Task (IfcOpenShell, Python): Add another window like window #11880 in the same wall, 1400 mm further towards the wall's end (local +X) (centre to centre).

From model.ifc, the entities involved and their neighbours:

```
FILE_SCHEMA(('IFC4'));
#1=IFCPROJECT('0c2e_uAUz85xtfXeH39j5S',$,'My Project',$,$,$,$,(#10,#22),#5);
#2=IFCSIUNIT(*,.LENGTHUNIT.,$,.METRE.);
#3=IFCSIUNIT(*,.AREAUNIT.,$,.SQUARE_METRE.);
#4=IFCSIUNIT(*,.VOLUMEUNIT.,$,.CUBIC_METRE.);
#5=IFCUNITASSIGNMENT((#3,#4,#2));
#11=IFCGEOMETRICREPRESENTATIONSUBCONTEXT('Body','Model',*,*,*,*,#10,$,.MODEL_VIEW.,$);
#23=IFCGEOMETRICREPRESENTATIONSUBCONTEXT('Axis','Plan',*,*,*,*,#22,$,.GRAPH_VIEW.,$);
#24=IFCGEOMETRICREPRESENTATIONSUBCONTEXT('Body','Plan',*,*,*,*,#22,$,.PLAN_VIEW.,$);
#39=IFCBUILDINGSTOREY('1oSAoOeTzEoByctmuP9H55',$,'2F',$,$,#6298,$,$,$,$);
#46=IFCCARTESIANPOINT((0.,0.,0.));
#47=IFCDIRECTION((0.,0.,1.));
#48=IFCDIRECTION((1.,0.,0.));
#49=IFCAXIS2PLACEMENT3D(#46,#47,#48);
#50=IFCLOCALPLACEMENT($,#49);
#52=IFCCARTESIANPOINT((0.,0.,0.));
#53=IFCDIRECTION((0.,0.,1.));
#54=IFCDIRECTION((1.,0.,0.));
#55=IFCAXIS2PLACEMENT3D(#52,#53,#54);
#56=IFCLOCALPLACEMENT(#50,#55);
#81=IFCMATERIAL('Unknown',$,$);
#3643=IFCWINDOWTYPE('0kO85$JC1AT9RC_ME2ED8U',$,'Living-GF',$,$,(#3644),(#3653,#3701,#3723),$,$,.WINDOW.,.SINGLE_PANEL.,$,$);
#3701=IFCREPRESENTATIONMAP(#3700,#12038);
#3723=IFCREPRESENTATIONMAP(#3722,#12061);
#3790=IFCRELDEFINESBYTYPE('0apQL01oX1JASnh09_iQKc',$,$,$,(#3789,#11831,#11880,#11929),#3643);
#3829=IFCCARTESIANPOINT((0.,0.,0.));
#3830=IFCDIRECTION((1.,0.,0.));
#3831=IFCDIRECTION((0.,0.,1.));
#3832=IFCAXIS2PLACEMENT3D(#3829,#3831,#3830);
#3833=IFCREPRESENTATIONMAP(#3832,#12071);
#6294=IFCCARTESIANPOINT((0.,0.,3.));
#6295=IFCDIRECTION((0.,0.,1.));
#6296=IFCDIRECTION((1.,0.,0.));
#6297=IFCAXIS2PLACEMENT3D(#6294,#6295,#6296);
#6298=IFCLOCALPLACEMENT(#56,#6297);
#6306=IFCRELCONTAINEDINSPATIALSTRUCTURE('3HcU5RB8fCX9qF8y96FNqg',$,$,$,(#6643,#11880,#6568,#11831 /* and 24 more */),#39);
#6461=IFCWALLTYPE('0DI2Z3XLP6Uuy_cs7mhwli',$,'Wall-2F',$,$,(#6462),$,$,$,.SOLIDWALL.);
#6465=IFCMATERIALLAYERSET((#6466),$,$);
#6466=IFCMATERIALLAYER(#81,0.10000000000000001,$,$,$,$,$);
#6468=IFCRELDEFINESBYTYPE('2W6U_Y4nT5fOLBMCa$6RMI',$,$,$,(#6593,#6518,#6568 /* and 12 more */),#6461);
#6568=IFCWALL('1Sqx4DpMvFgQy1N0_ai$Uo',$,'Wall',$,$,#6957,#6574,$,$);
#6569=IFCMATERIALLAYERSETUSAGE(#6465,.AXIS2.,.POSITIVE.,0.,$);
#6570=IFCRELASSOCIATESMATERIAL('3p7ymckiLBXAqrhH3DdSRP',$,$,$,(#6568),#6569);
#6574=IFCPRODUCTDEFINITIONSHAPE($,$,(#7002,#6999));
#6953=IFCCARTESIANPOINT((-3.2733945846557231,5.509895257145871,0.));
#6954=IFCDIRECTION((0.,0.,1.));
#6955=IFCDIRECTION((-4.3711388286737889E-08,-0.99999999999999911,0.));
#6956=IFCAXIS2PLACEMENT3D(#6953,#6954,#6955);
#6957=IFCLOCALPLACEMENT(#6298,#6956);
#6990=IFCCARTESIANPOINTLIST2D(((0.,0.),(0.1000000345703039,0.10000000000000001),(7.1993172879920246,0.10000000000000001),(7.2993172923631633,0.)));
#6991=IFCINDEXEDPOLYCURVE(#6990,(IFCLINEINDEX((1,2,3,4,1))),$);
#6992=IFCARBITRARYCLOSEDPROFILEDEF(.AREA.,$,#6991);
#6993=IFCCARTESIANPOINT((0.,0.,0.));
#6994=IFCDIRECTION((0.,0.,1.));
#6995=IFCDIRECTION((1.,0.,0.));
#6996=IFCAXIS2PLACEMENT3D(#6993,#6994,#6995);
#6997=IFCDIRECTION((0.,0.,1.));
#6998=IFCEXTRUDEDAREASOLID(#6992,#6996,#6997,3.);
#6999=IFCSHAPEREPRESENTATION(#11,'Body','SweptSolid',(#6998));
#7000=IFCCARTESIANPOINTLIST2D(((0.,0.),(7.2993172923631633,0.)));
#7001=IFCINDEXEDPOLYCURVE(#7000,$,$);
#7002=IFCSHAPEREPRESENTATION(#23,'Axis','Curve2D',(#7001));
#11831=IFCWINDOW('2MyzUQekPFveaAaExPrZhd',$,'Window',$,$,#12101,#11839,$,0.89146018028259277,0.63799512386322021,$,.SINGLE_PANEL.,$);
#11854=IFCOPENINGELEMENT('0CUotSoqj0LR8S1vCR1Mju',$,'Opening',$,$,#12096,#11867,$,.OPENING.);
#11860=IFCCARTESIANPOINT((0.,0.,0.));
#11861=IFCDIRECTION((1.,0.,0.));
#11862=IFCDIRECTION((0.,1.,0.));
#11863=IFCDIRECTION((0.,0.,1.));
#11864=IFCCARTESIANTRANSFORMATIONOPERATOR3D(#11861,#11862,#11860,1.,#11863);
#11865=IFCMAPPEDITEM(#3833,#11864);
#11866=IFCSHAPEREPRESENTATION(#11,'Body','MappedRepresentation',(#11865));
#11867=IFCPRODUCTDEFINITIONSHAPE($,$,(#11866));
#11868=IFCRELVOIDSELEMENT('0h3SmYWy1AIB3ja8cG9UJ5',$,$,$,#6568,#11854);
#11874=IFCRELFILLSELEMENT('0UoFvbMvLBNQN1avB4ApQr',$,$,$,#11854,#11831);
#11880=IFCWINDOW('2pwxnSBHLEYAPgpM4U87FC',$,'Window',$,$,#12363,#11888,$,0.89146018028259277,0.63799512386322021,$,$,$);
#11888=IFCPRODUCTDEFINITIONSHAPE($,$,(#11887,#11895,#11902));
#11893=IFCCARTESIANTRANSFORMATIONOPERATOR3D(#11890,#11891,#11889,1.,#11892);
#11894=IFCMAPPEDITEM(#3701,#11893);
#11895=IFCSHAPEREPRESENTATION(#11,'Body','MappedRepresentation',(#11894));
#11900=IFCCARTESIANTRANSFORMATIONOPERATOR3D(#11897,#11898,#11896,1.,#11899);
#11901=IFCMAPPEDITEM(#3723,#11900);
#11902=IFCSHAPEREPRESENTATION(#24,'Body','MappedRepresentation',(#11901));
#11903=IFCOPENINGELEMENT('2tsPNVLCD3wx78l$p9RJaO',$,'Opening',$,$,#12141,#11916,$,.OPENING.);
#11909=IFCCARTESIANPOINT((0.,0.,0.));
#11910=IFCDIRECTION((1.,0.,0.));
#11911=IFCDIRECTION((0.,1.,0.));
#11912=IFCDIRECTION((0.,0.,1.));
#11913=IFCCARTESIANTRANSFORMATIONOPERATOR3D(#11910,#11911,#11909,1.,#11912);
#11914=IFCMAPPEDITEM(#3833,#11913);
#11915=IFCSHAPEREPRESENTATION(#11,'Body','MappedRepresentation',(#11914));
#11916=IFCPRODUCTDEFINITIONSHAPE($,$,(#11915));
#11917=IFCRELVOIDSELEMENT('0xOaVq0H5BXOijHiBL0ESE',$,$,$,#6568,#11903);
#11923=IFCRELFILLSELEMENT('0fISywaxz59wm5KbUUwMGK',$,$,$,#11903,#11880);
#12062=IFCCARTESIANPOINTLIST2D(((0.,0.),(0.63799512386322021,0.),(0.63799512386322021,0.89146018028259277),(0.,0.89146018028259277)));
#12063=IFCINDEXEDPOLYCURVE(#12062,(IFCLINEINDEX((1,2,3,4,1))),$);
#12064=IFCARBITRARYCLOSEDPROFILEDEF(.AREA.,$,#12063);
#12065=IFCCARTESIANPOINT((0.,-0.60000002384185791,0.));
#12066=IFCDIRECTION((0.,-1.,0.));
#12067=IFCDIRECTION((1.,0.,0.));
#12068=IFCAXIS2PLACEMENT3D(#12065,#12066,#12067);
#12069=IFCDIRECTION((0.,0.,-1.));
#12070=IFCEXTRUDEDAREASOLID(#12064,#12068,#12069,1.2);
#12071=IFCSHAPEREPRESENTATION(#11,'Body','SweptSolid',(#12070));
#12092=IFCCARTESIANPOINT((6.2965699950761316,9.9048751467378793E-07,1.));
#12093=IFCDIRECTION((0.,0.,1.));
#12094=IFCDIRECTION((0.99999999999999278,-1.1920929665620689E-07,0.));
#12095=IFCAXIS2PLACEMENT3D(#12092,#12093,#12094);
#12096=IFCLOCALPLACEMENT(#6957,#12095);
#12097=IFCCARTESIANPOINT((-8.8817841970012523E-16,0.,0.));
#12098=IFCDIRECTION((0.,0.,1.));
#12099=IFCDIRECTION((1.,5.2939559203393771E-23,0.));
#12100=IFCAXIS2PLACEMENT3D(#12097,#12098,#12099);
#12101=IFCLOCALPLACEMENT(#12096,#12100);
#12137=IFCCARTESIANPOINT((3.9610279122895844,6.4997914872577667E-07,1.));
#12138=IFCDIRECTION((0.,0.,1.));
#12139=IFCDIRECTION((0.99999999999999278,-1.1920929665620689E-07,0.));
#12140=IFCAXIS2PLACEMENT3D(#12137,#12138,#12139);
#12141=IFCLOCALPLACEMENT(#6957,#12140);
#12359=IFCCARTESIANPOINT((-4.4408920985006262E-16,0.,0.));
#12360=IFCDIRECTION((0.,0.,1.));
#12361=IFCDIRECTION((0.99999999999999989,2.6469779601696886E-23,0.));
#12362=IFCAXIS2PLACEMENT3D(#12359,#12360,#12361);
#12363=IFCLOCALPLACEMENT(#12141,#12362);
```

```python
import ifcopenshell
import ifcopenshell.api.feature
import ifcopenshell.api.geometry
import ifcopenshell.api.root
import ifcopenshell.geom
import ifcopenshell.util.element
import ifcopenshell.util.placement
import ifcopenshell.util.shape
import ifcopenshell.util.unit

model = ifcopenshell.open("model.ifc")
unit_scale = ifcopenshell.util.unit.calculate_unit_scale(model)
settings = ifcopenshell.geom.settings()


def volume(element):
    """Net volume in cubic metres, openings subtracted."""
    shape = ifcopenshell.geom.create_shape(settings, element)
    return ifcopenshell.util.shape.get_volume(shape.geometry)


window = model.by_guid("2pwxnSBHLEYAPgpM4U87FC")
opening = window.FillsVoids[0].RelatingOpeningElement
wall = opening.VoidsElements[0].RelatingBuildingElement
before = volume(wall)
shift = ifcopenshell.util.placement.get_local_placement(wall.ObjectPlacement)[:3, 0] * 1.4 / unit_scale

# copy_class copies the void relationship, type, container and properties, but no geometry.
new_opening = ifcopenshell.api.root.copy_class(model, product=opening)
new_opening.Representation = ifcopenshell.util.element.copy_deep(
    model, opening.Representation, exclude=["IfcGeometricRepresentationContext", "IfcRepresentationMap"]
)
new_window = ifcopenshell.api.root.copy_class(model, product=window)
new_window.Representation = ifcopenshell.util.element.copy_deep(
    model, window.Representation, exclude=["IfcGeometricRepresentationContext", "IfcRepresentationMap"]
)
ifcopenshell.api.feature.add_filling(model, opening=new_opening, element=new_window)

for old, new in ((opening, new_opening), (window, new_window)):
    matrix = ifcopenshell.util.placement.get_local_placement(old.ObjectPlacement)
    matrix[:3, 3] += shift
    ifcopenshell.api.geometry.edit_object_placement(model, product=new, matrix=matrix, is_si=False)

after = volume(wall)

print(f"wall volume {before:.3f} -> {after:.3f} m3")

model.write("model_edited.ifc")
```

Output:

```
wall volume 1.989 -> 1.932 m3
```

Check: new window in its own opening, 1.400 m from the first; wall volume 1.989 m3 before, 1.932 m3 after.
